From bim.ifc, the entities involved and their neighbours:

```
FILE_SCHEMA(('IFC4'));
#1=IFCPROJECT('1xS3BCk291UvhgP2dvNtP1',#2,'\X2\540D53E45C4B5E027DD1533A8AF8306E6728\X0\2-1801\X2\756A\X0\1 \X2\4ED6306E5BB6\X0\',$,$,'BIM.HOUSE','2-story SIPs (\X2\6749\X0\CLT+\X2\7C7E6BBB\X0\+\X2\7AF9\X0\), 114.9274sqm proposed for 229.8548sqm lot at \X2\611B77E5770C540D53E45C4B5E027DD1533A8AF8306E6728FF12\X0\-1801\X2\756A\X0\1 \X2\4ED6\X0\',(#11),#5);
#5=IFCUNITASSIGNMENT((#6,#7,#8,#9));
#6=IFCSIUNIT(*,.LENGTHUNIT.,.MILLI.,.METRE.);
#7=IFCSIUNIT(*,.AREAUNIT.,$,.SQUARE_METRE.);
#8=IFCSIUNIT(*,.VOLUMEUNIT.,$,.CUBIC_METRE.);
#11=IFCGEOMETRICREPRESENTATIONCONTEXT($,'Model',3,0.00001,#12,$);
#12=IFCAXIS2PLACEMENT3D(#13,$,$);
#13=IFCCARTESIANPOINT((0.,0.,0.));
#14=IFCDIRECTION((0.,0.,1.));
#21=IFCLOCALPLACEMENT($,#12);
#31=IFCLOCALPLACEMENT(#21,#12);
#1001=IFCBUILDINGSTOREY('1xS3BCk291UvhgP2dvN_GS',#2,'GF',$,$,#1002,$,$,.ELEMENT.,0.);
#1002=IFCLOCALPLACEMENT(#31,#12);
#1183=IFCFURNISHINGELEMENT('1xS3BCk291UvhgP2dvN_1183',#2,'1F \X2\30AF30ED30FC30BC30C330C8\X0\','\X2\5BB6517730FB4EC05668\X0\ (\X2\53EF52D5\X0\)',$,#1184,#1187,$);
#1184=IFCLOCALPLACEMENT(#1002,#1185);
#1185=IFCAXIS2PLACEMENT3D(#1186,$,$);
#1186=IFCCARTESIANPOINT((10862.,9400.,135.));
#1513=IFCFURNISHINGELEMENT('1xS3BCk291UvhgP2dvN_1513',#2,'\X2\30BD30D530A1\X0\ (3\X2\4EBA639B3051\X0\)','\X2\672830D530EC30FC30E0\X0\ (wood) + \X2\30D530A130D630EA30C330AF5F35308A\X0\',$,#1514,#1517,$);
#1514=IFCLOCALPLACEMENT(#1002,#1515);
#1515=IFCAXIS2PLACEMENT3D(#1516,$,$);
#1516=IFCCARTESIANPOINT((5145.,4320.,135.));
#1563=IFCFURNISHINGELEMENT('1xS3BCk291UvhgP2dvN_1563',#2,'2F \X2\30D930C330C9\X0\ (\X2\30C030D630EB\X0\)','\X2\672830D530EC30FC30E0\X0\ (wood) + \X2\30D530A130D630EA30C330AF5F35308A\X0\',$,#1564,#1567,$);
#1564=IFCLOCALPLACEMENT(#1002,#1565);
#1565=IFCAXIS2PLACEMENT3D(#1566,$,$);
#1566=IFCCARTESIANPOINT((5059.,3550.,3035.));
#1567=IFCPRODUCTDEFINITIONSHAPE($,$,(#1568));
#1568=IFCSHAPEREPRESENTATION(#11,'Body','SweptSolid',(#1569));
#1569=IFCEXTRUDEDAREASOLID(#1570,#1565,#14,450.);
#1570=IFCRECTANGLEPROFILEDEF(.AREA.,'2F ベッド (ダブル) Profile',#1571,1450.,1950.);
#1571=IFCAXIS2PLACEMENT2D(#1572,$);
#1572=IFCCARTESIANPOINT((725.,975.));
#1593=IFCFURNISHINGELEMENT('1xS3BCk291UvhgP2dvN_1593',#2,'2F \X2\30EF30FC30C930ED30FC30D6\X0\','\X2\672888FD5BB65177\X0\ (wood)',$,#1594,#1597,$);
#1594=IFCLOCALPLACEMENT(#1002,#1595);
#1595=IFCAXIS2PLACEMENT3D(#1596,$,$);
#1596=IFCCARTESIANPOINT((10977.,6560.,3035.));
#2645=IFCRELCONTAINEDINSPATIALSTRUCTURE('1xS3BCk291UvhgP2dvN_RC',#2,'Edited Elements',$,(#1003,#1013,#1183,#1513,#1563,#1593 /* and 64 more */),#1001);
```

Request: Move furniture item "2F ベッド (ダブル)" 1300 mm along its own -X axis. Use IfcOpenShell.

```python
import ifcopenshell
import ifcopenshell.api.geometry
import ifcopenshell.util.placement
import ifcopenshell.util.unit

model = ifcopenshell.open("bim.ifc")
unit_scale = ifcopenshell.util.unit.calculate_unit_scale(model)

item = model.by_guid("1xS3BCk291UvhgP2dvN_1563")
matrix = ifcopenshell.util.placement.get_local_placement(item.ObjectPlacement)
matrix[:3, 3] -= matrix[:3, 0] * 1.3 / unit_scale
ifcopenshell.api.geometry.edit_object_placement(model, product=item, matrix=matrix, is_si=False)

print(ifcopenshell.util.placement.get_local_placement(item.ObjectPlacement).round(3) + 0.0)

model.write("bim_edited.ifc")
```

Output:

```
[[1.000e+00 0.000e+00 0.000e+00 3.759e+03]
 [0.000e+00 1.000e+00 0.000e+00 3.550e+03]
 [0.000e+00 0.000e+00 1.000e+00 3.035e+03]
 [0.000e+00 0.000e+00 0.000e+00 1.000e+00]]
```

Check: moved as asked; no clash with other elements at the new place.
